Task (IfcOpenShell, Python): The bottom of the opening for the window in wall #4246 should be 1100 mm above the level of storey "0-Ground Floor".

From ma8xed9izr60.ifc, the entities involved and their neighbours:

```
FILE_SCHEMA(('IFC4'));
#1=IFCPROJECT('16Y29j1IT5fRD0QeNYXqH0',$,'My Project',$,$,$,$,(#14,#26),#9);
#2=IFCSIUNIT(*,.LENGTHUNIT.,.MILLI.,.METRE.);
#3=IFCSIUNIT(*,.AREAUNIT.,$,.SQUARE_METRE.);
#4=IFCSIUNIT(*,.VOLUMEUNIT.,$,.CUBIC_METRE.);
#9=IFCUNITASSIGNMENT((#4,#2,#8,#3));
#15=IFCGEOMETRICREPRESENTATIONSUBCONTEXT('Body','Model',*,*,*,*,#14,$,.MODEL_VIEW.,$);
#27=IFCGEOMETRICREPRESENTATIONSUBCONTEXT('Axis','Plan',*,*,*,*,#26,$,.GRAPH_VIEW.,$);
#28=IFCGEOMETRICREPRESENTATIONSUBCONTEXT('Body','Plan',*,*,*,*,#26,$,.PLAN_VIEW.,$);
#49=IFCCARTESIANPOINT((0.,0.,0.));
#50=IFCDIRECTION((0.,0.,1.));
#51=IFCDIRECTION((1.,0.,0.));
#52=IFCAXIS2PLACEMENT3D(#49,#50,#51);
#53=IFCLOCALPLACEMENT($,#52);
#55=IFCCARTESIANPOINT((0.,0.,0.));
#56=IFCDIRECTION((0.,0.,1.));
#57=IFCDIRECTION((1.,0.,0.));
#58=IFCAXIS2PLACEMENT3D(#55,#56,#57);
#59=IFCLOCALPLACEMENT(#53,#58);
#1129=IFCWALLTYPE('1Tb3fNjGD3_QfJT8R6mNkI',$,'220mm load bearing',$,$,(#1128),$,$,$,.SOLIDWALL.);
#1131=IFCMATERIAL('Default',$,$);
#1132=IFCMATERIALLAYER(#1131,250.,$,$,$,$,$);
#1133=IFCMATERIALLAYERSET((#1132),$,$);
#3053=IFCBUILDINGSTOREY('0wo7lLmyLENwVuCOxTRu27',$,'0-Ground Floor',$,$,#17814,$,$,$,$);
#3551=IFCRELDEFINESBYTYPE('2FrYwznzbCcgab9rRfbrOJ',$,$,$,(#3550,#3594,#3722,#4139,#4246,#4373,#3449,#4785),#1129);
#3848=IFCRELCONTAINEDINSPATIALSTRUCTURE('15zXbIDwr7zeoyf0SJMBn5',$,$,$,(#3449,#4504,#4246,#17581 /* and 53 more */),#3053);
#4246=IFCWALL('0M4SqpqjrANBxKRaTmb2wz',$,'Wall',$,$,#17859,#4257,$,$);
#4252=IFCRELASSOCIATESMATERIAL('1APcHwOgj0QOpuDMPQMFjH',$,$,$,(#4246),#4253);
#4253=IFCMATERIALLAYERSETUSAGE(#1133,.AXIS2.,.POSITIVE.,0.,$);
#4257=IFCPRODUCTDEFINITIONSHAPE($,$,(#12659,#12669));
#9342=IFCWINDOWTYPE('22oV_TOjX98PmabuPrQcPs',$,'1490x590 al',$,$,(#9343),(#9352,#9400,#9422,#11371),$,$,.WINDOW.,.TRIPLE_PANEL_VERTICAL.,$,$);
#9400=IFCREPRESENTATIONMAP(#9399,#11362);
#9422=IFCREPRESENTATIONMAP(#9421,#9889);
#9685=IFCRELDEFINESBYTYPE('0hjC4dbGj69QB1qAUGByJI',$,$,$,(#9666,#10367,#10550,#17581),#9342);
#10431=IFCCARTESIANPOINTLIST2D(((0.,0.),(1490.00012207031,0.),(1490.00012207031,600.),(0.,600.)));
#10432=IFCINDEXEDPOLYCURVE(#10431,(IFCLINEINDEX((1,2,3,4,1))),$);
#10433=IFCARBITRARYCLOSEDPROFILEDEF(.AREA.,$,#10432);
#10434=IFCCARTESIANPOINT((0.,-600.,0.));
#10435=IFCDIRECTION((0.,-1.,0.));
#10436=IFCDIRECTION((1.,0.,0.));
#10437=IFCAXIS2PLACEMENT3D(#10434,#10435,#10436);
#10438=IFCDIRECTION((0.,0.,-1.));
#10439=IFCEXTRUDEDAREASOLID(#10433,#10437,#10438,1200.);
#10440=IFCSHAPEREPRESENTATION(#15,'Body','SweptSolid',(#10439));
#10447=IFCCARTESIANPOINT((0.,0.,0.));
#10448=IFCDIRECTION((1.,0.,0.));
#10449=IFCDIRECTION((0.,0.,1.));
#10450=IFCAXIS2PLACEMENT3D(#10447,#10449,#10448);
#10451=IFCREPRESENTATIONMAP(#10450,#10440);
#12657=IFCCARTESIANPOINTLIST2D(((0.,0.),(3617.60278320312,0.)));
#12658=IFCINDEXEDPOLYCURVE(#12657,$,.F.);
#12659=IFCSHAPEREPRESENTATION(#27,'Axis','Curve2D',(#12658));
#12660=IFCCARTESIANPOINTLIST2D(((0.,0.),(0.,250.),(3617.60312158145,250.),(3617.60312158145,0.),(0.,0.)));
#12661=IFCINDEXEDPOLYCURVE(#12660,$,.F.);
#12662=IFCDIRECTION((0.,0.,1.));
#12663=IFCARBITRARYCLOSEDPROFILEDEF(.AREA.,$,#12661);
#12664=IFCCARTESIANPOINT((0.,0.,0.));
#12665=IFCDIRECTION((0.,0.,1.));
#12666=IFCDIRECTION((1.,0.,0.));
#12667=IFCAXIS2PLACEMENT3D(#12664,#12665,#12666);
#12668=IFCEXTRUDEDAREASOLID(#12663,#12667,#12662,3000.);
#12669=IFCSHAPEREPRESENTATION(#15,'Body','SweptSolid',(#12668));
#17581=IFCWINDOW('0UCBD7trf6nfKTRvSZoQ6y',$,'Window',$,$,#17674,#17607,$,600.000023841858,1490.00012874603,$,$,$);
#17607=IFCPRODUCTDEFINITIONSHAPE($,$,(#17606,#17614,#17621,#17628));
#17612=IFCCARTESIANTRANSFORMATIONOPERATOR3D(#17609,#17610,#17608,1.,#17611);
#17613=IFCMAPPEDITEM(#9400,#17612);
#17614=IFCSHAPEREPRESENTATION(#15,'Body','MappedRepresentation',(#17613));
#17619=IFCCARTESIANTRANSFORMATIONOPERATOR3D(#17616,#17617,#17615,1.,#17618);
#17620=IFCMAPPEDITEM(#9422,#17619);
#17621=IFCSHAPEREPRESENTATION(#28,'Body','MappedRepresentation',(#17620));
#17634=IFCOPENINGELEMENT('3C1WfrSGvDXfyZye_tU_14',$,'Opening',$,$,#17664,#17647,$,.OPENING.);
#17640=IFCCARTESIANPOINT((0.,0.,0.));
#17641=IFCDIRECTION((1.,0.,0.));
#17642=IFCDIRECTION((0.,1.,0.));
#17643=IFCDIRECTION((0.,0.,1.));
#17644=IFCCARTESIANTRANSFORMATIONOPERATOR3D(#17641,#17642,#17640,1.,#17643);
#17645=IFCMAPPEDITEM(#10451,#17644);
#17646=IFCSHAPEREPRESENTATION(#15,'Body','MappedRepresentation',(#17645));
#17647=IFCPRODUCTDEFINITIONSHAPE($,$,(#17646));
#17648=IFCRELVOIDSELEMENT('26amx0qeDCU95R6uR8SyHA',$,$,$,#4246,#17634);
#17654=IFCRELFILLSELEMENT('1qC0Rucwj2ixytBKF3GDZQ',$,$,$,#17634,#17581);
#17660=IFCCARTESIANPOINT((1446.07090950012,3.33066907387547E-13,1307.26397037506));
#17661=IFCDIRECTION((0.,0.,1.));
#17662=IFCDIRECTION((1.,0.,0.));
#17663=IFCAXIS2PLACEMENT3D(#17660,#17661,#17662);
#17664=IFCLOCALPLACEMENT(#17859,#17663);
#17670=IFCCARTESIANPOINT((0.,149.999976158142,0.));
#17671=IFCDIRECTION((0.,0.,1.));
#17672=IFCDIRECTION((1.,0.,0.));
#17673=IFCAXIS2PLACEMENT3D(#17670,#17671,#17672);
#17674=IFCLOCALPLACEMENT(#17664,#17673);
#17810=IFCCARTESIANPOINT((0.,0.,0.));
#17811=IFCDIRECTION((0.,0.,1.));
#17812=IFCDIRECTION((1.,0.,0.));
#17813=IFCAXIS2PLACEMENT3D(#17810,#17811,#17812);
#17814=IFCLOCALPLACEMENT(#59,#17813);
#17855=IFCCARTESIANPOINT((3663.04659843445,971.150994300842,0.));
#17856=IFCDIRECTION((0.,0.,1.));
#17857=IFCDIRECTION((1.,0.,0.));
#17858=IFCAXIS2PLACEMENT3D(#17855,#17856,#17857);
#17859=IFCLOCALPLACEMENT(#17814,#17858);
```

```python
import numpy as np
import ifcopenshell
import ifcopenshell.api.geometry
import ifcopenshell.geom
import ifcopenshell.util.element
import ifcopenshell.util.placement
import ifcopenshell.util.shape
import ifcopenshell.util.unit

model = ifcopenshell.open("ma8xed9izr60.ifc")
unit_scale = ifcopenshell.util.unit.calculate_unit_scale(model)

window = model.by_id(17581)
opening = window.FillsVoids[0].RelatingOpeningElement
storey = ifcopenshell.util.element.get_container(window, ifc_class="IfcBuildingStorey")
level = ifcopenshell.util.placement.get_local_placement(storey.ObjectPlacement)[2, 3]

# The opening's origin need not be at the sill, so measure its lowest point.
shape = ifcopenshell.geom.create_shape(ifcopenshell.geom.settings(), opening)
bottom = ifcopenshell.util.shape.get_shape_bottom_elevation(shape, shape.geometry) / unit_scale
dz = level + 1100.0 - bottom

shift = np.array([0.0, 0.0, dz])
# The window is placed relative to its opening, so it follows when the opening moves.
matrix = ifcopenshell.util.placement.get_local_placement(opening.ObjectPlacement)
matrix[:3, 3] += shift
ifcopenshell.api.geometry.edit_object_placement(
    model, product=opening, matrix=matrix, is_si=False, should_transform_children=True
)

print(f"moved by {dz * unit_scale:+.3f} m")

model.write("ma8xed9izr60-out.ifc")
```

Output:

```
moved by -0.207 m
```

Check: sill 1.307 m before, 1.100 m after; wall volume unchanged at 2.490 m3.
